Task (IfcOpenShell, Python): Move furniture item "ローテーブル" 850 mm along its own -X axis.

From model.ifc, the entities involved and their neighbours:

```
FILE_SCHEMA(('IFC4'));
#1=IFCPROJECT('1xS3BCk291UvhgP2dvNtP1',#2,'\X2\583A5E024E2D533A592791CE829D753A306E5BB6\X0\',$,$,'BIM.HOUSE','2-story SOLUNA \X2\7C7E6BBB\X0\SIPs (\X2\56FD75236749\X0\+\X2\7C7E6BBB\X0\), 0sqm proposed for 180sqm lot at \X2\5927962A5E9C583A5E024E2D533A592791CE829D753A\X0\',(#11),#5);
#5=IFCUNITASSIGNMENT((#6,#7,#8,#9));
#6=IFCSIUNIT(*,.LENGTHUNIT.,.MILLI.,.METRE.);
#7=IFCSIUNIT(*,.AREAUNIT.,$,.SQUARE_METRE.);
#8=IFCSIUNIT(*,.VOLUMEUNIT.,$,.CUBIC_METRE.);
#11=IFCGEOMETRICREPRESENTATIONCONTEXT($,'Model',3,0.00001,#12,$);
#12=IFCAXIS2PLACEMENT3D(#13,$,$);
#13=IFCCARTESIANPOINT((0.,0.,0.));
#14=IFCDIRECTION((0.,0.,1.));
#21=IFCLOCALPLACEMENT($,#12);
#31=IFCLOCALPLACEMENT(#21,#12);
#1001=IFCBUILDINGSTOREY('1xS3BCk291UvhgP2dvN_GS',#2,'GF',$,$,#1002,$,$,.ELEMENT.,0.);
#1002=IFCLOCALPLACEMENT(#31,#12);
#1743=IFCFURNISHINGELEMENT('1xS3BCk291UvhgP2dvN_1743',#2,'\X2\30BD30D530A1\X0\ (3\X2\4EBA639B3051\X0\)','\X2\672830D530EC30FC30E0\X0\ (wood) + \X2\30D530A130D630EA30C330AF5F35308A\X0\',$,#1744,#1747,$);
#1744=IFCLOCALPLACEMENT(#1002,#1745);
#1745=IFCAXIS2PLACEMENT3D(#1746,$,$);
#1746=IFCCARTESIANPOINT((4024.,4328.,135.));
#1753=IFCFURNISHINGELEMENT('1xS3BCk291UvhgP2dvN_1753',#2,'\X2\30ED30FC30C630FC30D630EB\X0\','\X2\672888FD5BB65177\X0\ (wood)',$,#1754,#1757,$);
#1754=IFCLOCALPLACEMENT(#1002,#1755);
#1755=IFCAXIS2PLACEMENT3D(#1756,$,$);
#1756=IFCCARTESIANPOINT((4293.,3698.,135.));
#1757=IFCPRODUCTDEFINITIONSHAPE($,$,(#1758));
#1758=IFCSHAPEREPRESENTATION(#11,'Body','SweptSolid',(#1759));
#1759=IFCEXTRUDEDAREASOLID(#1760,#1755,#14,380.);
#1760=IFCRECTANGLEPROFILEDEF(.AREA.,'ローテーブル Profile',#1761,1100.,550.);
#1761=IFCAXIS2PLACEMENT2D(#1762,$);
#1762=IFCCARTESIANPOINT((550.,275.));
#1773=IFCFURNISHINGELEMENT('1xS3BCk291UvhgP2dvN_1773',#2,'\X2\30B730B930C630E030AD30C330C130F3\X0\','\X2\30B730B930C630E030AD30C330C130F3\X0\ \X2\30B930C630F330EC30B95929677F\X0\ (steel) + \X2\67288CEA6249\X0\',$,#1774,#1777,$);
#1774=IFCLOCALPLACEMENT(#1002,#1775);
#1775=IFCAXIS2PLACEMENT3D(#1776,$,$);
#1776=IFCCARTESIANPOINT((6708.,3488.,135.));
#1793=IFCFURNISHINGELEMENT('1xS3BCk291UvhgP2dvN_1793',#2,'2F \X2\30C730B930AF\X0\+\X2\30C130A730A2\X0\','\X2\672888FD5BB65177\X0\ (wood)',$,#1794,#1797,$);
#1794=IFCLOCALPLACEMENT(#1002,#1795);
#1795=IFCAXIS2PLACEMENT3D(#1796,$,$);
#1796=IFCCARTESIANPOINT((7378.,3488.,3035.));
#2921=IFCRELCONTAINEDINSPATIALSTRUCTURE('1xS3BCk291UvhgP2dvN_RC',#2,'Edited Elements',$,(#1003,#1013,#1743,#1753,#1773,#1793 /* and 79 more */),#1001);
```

```python
import ifcopenshell
import ifcopenshell.api.geometry
import ifcopenshell.util.placement
import ifcopenshell.util.unit

model = ifcopenshell.open("model.ifc")
unit_scale = ifcopenshell.util.unit.calculate_unit_scale(model)

item = model.by_guid("1xS3BCk291UvhgP2dvN_1753")
matrix = ifcopenshell.util.placement.get_local_placement(item.ObjectPlacement)
matrix[:3, 3] -= matrix[:3, 0] * 0.85 / unit_scale
ifcopenshell.api.geometry.edit_object_placement(model, product=item, matrix=matrix, is_si=False)

print(ifcopenshell.util.placement.get_local_placement(item.ObjectPlacement).round(3) + 0.0)

model.write("model_edited.ifc")
```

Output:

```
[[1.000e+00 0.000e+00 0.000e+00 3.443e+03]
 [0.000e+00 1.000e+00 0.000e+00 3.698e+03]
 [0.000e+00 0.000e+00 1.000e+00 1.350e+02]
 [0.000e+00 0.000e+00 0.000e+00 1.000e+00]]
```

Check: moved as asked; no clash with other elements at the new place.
